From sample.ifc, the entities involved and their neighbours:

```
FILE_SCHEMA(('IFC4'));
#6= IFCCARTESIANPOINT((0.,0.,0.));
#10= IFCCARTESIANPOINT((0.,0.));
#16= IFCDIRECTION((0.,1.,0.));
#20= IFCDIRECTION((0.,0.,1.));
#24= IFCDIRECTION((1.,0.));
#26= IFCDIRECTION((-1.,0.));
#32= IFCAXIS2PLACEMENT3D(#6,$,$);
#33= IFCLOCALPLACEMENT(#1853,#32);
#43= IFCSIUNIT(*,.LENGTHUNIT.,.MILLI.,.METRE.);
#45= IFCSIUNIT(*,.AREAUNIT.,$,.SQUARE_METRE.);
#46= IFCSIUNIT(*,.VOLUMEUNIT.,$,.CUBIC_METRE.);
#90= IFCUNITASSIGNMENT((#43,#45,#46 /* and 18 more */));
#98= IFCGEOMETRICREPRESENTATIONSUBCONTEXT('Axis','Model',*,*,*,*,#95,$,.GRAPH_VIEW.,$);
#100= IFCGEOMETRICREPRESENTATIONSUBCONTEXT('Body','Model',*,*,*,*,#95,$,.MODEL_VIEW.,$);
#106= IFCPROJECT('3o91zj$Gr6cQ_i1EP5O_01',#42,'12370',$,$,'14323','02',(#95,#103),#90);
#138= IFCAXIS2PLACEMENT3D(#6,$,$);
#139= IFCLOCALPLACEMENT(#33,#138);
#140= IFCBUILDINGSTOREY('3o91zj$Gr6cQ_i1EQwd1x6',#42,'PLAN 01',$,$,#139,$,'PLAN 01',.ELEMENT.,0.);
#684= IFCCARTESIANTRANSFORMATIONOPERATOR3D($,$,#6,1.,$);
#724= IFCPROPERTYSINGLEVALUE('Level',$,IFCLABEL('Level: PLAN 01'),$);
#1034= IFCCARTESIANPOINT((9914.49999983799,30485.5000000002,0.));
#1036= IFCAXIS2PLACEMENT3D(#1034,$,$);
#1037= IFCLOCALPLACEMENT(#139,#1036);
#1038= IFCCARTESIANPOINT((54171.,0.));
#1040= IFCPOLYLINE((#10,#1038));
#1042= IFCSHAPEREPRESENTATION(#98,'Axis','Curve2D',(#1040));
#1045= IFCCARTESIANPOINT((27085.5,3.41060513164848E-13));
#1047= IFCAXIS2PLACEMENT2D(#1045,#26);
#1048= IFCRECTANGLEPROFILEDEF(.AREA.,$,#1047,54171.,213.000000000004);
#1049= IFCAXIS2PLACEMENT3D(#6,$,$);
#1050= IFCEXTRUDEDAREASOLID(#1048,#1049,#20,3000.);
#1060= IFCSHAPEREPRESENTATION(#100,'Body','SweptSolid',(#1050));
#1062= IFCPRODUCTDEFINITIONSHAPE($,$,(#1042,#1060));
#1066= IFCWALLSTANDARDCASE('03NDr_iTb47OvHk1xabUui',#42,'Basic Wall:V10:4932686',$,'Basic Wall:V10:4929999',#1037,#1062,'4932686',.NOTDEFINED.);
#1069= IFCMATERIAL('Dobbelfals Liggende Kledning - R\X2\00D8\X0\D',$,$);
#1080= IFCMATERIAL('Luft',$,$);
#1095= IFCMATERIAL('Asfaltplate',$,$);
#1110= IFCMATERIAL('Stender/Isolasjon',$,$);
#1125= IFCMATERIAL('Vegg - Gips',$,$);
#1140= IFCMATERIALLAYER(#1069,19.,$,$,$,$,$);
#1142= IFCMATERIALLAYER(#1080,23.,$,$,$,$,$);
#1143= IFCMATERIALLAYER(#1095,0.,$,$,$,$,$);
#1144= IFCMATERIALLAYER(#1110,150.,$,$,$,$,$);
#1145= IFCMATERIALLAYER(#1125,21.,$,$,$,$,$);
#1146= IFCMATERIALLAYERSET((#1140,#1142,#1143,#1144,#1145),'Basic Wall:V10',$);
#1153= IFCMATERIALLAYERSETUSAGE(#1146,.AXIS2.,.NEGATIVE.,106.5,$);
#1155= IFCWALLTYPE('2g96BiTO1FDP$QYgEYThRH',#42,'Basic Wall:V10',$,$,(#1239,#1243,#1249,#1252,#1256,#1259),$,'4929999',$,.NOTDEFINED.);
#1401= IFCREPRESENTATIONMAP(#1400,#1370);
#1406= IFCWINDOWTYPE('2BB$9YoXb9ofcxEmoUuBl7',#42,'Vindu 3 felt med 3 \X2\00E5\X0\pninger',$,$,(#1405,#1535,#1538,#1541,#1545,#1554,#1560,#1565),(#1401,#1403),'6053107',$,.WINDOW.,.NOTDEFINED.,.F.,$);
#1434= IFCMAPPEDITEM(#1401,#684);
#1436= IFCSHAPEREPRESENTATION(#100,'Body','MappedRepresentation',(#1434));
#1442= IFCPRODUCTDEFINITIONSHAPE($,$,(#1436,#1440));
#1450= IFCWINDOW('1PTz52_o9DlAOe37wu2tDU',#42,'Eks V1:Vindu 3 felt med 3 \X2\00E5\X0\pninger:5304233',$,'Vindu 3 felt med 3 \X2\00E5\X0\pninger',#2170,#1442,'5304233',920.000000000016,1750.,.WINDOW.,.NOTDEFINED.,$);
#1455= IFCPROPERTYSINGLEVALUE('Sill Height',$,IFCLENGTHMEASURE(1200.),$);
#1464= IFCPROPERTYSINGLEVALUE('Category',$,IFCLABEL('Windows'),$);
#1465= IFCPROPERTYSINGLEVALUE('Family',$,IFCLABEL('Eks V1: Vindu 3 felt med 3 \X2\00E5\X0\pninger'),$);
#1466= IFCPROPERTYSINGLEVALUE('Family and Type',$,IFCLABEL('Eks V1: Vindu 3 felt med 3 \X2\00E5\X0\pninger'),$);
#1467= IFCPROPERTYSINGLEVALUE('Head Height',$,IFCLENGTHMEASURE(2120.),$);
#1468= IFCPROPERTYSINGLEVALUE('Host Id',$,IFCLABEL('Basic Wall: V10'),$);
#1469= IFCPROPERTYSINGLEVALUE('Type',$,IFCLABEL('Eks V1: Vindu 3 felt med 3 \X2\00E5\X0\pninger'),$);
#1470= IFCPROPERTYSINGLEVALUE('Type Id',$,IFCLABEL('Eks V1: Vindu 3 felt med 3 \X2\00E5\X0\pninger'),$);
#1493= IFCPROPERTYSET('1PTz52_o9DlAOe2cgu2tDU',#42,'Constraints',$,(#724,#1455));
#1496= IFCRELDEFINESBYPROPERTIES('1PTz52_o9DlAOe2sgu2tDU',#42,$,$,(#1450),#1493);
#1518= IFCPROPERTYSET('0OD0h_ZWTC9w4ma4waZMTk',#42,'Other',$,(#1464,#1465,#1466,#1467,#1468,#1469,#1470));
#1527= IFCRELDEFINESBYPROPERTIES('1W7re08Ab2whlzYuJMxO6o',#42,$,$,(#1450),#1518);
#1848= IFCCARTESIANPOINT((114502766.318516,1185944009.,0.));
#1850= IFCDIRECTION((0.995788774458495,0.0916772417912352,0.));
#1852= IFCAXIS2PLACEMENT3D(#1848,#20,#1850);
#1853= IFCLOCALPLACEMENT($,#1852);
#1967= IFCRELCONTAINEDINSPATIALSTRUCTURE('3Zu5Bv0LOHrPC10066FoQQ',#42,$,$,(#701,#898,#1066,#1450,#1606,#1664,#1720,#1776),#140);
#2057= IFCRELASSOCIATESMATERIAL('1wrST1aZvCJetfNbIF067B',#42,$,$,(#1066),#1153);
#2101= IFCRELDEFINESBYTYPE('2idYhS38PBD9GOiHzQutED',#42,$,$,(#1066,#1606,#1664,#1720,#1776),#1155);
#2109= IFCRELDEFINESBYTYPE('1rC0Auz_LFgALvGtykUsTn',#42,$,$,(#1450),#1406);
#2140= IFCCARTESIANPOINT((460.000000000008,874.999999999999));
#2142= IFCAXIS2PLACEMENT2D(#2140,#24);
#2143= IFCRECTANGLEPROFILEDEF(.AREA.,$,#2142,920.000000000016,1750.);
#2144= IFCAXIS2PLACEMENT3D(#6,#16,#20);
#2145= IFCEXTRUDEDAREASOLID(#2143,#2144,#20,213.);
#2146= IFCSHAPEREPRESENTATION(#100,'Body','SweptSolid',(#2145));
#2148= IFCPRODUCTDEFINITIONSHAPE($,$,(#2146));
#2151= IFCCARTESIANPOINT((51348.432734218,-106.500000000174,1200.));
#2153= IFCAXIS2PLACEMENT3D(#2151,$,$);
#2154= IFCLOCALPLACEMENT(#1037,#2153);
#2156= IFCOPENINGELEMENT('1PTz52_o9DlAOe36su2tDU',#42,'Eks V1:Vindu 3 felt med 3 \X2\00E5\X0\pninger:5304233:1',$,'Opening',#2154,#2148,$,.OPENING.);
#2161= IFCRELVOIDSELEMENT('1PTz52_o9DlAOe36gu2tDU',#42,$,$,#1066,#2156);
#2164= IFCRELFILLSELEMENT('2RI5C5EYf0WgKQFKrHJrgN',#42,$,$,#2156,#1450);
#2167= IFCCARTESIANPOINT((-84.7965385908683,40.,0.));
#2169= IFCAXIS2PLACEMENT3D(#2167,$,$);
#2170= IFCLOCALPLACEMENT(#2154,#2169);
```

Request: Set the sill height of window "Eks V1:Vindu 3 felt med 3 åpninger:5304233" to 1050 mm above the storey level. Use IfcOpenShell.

```python
import numpy as np
import ifcopenshell
import ifcopenshell.api.geometry
import ifcopenshell.api.pset
import ifcopenshell.geom
import ifcopenshell.util.element
import ifcopenshell.util.placement
import ifcopenshell.util.shape
import ifcopenshell.util.unit

model = ifcopenshell.open("sample.ifc")
unit_scale = ifcopenshell.util.unit.calculate_unit_scale(model)

window = model.by_guid("1PTz52_o9DlAOe37wu2tDU")
opening = window.FillsVoids[0].RelatingOpeningElement
storey = ifcopenshell.util.element.get_container(window, ifc_class="IfcBuildingStorey")
level = ifcopenshell.util.placement.get_local_placement(storey.ObjectPlacement)[2, 3]

# The opening's origin need not be at the sill, so measure its lowest point.
shape = ifcopenshell.geom.create_shape(ifcopenshell.geom.settings(), opening)
bottom = ifcopenshell.util.shape.get_shape_bottom_elevation(shape, shape.geometry) / unit_scale
dz = level + 1050.0 - bottom

shift = np.array([0.0, 0.0, dz])
# The window is placed relative to its opening, so it follows when the opening moves.
matrix = ifcopenshell.util.placement.get_local_placement(opening.ObjectPlacement)
matrix[:3, 3] += shift
ifcopenshell.api.geometry.edit_object_placement(
    model, product=opening, matrix=matrix, is_si=False, should_transform_children=True
)

# Keep the stored heights in step.
pset = model.by_id(ifcopenshell.util.element.get_pset(window, "Constraints", should_inherit=False)["id"])
ifcopenshell.api.pset.edit_pset(model, pset=pset, properties={
    "Sill Height": model.create_entity("IfcLengthMeasure", ifcopenshell.util.element.get_pset(window, "Constraints", "Sill Height") + dz),
})
pset = model.by_id(ifcopenshell.util.element.get_pset(window, "Other", should_inherit=False)["id"])
ifcopenshell.api.pset.edit_pset(model, pset=pset, properties={
    "Head Height": model.create_entity("IfcLengthMeasure", ifcopenshell.util.element.get_pset(window, "Other", "Head Height") + dz),
})

print(f"moved by {dz * unit_scale:+.3f} m")

model.write("sample_edited.ifc")
```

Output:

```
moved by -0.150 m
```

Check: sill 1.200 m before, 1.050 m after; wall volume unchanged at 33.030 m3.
